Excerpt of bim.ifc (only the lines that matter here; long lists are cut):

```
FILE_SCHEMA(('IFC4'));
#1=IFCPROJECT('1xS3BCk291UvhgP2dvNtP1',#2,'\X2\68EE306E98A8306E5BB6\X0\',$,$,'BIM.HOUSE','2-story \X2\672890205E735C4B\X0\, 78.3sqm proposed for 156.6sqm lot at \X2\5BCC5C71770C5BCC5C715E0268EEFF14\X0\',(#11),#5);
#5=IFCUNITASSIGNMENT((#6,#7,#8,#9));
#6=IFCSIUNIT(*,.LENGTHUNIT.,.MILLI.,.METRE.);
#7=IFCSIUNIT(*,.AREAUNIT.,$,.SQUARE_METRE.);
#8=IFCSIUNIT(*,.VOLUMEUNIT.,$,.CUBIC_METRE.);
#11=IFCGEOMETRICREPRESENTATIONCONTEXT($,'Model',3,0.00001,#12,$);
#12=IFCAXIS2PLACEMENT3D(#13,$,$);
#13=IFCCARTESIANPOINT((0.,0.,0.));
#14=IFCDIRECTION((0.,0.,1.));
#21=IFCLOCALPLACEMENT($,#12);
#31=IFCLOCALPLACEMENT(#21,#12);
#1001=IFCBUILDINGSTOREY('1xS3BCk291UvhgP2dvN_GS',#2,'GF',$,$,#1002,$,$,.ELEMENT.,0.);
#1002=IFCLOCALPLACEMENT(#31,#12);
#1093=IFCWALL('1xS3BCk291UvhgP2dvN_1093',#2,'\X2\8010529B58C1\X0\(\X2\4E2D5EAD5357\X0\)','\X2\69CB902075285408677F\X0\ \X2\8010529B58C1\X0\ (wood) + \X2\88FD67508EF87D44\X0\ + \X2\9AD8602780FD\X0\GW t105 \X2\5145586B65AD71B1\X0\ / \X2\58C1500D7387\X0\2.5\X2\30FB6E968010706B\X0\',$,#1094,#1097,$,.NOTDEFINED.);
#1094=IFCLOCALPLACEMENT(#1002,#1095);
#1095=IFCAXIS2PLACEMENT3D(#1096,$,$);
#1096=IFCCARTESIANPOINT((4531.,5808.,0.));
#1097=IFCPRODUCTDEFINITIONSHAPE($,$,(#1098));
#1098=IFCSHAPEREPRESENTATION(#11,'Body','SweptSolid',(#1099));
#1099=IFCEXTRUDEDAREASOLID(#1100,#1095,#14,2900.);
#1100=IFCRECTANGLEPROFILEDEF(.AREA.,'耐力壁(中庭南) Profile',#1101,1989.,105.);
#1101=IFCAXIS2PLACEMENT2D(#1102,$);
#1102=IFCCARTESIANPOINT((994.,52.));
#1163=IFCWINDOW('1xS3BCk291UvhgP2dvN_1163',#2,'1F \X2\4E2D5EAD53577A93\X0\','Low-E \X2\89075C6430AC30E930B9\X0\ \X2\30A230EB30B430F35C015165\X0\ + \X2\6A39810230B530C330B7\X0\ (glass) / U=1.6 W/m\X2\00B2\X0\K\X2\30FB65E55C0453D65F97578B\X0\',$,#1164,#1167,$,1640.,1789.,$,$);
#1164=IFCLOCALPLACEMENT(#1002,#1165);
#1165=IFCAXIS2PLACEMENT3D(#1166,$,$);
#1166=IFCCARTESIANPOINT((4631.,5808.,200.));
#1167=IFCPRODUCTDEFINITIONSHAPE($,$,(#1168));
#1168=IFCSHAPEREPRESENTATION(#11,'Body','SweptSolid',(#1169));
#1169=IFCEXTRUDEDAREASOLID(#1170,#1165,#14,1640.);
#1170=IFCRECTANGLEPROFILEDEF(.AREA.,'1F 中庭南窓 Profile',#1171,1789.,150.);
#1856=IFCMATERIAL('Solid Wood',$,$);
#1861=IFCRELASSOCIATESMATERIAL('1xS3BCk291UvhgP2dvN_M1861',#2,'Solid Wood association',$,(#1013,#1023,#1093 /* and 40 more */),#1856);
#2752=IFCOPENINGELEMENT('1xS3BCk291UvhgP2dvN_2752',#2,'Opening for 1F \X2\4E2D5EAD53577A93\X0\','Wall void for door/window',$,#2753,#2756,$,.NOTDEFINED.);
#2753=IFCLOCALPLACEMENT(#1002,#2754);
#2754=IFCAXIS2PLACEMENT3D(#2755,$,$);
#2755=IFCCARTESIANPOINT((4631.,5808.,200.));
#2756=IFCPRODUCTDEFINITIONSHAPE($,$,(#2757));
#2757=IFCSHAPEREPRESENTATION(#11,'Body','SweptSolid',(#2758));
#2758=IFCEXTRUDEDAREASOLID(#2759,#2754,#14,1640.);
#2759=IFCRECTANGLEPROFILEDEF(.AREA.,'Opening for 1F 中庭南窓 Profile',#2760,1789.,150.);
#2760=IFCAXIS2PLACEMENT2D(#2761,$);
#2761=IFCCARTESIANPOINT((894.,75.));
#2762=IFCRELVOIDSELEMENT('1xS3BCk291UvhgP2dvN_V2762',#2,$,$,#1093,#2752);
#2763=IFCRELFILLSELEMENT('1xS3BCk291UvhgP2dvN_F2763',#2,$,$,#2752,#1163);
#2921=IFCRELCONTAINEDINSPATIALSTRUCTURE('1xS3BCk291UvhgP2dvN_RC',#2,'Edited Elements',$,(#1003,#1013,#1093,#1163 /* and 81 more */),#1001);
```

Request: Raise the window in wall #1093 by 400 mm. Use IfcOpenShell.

```python
import numpy as np
import ifcopenshell
import ifcopenshell.api.geometry
import ifcopenshell.util.placement
import ifcopenshell.util.unit

model = ifcopenshell.open("bim.ifc")
unit_scale = ifcopenshell.util.unit.calculate_unit_scale(model)

window = model.by_guid("1xS3BCk291UvhgP2dvN_1163")
opening = window.FillsVoids[0].RelatingOpeningElement
dz = 0.4 / unit_scale

shift = np.array([0.0, 0.0, dz])
# The window is not placed relative to its opening, so move both.
for product in (opening, window):
    matrix = ifcopenshell.util.placement.get_local_placement(product.ObjectPlacement)
    matrix[:3, 3] += shift
    ifcopenshell.api.geometry.edit_object_placement(model, product=product, matrix=matrix, is_si=False)

print(f"moved by {dz * unit_scale:+.3f} m")

model.write("bim_v2.ifc")
```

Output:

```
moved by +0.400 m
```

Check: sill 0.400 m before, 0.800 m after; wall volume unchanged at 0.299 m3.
